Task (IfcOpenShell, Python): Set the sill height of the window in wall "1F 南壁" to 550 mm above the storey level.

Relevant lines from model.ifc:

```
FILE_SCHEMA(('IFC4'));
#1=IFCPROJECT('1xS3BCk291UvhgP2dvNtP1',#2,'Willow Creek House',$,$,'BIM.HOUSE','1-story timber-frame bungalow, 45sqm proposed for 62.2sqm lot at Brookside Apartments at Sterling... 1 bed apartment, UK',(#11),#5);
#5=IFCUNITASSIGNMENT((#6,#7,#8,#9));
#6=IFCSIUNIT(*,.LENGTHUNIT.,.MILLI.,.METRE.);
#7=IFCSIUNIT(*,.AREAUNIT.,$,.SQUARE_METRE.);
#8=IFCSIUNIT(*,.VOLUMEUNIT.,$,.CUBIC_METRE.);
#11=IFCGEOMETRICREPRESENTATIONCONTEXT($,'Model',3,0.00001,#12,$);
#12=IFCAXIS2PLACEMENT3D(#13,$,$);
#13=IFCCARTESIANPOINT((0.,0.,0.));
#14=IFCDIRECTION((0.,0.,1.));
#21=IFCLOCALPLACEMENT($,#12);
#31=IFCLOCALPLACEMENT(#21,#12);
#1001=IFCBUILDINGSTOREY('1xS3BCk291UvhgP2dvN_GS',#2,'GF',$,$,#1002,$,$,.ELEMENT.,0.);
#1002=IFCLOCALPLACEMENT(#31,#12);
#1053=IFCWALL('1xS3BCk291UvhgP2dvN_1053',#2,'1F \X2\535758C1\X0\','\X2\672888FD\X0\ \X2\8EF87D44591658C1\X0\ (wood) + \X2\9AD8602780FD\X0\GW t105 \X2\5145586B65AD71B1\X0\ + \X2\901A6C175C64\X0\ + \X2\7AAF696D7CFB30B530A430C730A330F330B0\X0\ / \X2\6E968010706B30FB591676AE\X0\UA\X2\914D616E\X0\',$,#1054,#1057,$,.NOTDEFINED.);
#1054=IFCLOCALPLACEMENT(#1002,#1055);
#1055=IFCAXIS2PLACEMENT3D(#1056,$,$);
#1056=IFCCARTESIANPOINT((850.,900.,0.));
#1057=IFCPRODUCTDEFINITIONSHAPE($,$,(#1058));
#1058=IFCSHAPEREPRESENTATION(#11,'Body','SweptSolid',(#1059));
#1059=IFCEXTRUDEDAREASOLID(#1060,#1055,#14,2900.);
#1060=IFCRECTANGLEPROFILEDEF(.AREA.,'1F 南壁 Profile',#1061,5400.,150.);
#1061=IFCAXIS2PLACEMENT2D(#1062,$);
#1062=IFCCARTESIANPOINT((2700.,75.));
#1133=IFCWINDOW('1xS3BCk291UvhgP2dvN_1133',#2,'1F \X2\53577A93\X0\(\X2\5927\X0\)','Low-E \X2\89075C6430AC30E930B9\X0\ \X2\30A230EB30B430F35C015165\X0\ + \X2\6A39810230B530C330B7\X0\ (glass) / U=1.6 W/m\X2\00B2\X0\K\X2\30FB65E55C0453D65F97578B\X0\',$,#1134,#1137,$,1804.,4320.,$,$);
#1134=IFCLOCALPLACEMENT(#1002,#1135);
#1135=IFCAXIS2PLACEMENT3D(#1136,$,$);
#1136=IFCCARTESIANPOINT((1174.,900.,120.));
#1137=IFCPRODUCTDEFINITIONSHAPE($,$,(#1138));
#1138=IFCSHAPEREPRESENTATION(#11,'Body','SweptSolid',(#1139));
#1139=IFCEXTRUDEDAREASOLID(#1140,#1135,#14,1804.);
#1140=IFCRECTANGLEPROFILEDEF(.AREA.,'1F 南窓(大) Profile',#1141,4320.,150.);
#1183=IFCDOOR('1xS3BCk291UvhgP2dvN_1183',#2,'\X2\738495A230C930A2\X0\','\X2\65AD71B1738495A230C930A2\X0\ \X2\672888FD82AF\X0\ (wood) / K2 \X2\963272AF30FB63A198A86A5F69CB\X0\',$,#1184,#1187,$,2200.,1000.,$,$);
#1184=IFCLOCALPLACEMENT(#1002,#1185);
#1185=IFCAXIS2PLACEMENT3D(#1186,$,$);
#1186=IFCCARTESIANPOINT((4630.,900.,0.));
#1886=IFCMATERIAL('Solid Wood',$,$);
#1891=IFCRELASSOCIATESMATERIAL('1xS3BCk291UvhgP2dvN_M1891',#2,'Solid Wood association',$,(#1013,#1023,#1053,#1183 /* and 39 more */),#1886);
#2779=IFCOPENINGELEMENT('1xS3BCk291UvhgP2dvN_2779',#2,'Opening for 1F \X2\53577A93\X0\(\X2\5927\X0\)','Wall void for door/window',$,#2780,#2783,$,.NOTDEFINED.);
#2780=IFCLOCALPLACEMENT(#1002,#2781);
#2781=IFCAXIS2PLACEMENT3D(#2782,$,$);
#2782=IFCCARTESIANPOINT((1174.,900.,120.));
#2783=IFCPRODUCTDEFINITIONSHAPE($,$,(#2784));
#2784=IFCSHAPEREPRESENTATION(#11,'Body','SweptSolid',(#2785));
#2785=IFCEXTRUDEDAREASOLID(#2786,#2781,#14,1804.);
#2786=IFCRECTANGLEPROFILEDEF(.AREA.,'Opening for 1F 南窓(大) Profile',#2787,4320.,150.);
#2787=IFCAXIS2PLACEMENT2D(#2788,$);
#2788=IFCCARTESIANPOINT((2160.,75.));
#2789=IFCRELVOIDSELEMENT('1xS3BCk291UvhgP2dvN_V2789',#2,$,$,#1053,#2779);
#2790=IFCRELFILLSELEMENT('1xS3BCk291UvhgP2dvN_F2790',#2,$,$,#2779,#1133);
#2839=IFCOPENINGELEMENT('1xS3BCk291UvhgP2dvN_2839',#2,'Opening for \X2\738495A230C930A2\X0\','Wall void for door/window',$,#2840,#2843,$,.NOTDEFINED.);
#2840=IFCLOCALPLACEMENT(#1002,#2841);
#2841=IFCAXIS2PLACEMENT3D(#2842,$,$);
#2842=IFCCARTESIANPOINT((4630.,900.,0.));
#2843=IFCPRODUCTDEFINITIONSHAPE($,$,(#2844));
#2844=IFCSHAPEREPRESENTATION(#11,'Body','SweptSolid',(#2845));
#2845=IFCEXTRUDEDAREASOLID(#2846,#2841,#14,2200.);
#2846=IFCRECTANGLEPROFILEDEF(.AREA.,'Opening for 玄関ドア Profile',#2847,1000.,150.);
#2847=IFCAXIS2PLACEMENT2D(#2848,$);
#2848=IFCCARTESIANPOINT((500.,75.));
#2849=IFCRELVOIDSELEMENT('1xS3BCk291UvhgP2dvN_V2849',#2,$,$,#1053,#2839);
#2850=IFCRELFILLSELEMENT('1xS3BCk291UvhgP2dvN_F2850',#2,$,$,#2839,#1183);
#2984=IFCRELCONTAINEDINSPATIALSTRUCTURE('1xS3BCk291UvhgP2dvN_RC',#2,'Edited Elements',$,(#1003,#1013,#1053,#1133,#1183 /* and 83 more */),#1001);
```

```python
import numpy as np
import ifcopenshell
import ifcopenshell.api.geometry
import ifcopenshell.geom
import ifcopenshell.util.element
import ifcopenshell.util.placement
import ifcopenshell.util.shape
import ifcopenshell.util.unit

model = ifcopenshell.open("model.ifc")
unit_scale = ifcopenshell.util.unit.calculate_unit_scale(model)

window = model.by_guid("1xS3BCk291UvhgP2dvN_1133")
opening = window.FillsVoids[0].RelatingOpeningElement
storey = ifcopenshell.util.element.get_container(window, ifc_class="IfcBuildingStorey")
level = ifcopenshell.util.placement.get_local_placement(storey.ObjectPlacement)[2, 3]

# The opening's origin need not be at the sill, so measure its lowest point.
shape = ifcopenshell.geom.create_shape(ifcopenshell.geom.settings(), opening)
bottom = ifcopenshell.util.shape.get_shape_bottom_elevation(shape, shape.geometry) / unit_scale
dz = level + 550.0 - bottom

shift = np.array([0.0, 0.0, dz])
# The window is not placed relative to its opening, so move both.
for product in (opening, window):
    matrix = ifcopenshell.util.placement.get_local_placement(product.ObjectPlacement)
    matrix[:3, 3] += shift
    ifcopenshell.api.geometry.edit_object_placement(model, product=product, matrix=matrix, is_si=False)

print(f"moved by {dz * unit_scale:+.3f} m")

model.write("model-out.ifc")
```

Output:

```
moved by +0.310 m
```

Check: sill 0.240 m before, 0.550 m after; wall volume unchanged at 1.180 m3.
